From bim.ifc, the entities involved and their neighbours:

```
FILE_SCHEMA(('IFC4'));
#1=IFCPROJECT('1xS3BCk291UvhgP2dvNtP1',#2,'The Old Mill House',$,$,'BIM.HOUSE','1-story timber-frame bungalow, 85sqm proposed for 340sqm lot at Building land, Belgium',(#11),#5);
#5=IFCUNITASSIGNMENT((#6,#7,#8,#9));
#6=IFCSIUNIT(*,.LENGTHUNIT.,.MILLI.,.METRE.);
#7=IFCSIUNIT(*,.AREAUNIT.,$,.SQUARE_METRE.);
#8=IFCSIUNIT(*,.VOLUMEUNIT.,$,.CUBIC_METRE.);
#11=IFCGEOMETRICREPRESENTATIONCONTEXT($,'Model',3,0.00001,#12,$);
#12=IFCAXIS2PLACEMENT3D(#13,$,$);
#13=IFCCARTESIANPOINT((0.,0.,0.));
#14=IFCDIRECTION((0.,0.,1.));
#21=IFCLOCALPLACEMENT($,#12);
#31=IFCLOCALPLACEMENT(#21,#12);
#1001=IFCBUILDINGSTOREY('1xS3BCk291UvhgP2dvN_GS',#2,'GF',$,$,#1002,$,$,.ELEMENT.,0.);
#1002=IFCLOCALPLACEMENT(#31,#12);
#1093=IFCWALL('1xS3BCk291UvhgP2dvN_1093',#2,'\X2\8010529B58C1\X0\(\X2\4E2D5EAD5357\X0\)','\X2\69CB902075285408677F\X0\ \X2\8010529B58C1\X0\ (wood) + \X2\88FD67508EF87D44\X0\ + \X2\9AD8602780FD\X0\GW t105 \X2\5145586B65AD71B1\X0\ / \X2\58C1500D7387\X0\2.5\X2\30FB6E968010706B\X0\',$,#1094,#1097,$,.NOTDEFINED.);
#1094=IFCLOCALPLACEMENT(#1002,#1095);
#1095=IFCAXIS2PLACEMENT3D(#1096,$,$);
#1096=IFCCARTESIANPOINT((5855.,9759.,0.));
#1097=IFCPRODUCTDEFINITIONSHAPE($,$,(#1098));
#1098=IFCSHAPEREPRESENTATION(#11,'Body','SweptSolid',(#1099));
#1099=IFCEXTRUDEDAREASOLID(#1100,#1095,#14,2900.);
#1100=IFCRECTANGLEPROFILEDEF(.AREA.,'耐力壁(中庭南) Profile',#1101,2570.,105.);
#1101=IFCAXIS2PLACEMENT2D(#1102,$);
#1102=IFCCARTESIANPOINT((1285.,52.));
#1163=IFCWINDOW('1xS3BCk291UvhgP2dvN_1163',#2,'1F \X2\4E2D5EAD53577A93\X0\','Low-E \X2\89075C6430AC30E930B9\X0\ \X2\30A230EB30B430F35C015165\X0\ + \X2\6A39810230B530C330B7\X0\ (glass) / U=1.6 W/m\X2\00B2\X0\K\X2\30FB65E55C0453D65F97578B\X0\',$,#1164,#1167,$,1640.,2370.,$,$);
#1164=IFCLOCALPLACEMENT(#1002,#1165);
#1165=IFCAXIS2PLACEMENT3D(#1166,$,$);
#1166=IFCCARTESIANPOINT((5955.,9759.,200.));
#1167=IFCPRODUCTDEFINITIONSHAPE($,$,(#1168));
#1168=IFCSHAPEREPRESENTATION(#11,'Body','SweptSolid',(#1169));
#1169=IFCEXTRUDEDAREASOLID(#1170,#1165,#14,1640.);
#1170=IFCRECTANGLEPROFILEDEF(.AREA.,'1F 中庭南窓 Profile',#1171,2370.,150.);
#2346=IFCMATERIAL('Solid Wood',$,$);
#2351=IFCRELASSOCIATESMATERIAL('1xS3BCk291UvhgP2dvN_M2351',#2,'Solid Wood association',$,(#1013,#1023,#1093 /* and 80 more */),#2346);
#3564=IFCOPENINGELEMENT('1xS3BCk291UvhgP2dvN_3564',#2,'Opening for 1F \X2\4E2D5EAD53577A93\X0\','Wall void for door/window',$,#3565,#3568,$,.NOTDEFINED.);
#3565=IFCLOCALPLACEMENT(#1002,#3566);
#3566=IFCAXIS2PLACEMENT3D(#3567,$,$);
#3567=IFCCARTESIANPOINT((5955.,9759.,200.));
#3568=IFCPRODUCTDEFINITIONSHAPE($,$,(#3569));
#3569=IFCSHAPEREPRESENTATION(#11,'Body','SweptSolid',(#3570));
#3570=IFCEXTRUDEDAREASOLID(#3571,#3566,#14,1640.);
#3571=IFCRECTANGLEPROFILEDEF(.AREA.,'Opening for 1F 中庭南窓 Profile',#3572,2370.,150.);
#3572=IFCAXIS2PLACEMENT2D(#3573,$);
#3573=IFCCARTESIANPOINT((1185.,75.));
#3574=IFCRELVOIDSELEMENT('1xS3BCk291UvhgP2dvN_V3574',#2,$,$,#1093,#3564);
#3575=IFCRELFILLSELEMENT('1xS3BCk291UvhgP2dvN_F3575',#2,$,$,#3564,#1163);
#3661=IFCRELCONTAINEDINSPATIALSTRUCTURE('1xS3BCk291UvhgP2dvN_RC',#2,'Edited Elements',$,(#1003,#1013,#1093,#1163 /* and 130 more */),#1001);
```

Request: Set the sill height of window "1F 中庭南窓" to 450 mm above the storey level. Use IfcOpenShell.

```python
import numpy as np
import ifcopenshell
import ifcopenshell.api.geometry
import ifcopenshell.geom
import ifcopenshell.util.element
import ifcopenshell.util.placement
import ifcopenshell.util.shape
import ifcopenshell.util.unit

model = ifcopenshell.open("bim.ifc")
unit_scale = ifcopenshell.util.unit.calculate_unit_scale(model)

window = model.by_guid("1xS3BCk291UvhgP2dvN_1163")
opening = window.FillsVoids[0].RelatingOpeningElement
storey = ifcopenshell.util.element.get_container(window, ifc_class="IfcBuildingStorey")
level = ifcopenshell.util.placement.get_local_placement(storey.ObjectPlacement)[2, 3]

# The opening's origin need not be at the sill, so measure its lowest point.
shape = ifcopenshell.geom.create_shape(ifcopenshell.geom.settings(), opening)
bottom = ifcopenshell.util.shape.get_shape_bottom_elevation(shape, shape.geometry) / unit_scale
dz = level + 450.0 - bottom

shift = np.array([0.0, 0.0, dz])
# The window is not placed relative to its opening, so move both.
for product in (opening, window):
    matrix = ifcopenshell.util.placement.get_local_placement(product.ObjectPlacement)
    matrix[:3, 3] += shift
    ifcopenshell.api.geometry.edit_object_placement(model, product=product, matrix=matrix, is_si=False)

print(f"moved by {dz * unit_scale:+.3f} m")

model.write("bim_v2.ifc")
```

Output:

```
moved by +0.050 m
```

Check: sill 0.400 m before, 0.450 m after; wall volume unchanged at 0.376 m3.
